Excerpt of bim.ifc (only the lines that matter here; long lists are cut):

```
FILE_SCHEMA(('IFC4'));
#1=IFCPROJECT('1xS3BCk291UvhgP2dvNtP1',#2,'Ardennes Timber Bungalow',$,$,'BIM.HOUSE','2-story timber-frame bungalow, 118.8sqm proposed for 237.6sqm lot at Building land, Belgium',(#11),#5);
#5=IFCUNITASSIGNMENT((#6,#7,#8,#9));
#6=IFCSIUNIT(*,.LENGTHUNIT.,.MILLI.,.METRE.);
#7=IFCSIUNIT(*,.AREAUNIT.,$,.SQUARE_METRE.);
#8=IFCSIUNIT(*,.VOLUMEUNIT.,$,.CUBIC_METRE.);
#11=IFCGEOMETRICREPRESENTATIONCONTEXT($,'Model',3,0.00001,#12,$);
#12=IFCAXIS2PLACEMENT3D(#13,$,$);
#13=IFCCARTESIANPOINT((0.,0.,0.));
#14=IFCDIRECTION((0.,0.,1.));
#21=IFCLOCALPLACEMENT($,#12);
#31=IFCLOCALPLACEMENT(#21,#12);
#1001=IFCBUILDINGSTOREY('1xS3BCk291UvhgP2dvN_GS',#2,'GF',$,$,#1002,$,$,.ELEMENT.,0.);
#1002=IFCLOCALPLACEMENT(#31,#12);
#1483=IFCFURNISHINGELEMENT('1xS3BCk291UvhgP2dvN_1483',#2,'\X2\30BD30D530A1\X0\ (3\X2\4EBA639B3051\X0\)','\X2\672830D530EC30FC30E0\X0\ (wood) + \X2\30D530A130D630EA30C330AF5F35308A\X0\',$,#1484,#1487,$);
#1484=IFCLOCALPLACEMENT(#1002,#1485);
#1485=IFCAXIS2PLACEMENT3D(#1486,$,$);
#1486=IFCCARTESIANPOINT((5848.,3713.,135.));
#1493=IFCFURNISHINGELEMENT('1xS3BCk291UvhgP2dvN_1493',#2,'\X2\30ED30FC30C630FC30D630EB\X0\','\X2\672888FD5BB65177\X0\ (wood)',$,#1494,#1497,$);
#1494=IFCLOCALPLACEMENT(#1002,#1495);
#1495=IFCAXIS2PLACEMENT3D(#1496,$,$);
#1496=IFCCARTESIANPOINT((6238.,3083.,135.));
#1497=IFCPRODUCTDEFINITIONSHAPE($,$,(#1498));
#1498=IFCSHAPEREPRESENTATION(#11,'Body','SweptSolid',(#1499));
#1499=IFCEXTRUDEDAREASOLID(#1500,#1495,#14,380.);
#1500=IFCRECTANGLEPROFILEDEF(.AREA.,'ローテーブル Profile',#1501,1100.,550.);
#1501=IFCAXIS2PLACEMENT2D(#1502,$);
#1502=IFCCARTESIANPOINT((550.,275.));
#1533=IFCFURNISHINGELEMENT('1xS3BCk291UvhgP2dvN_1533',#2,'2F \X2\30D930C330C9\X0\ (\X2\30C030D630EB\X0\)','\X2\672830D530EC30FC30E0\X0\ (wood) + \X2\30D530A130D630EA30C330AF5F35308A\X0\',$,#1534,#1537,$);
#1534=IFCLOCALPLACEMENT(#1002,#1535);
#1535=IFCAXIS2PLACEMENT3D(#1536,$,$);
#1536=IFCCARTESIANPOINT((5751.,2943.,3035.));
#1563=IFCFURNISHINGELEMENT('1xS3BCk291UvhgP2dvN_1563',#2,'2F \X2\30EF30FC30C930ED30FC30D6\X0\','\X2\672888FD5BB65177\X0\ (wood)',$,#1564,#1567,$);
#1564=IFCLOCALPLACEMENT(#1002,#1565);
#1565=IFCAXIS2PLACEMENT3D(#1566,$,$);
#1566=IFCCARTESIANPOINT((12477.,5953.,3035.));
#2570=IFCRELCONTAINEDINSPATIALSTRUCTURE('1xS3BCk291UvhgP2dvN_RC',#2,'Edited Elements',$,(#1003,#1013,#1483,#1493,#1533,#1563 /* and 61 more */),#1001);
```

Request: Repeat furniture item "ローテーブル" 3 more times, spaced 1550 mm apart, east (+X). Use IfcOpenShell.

```python
import numpy as np
import ifcopenshell
import ifcopenshell.api.geometry
import ifcopenshell.api.root
import ifcopenshell.util.element
import ifcopenshell.util.placement
import ifcopenshell.util.unit

model = ifcopenshell.open("bim.ifc")
unit_scale = ifcopenshell.util.unit.calculate_unit_scale(model)


def reuse_history(source, copy):
    """copy_class also copies each property set's owner history, people and application; keep the originals."""
    for rel in copy.IsDefinedBy:
        if rel.is_a("IfcRelDefinesByProperties") and (history := rel.RelatingPropertyDefinition.OwnerHistory):
            rel.RelatingPropertyDefinition.OwnerHistory = source.OwnerHistory
            ifcopenshell.util.element.remove_deep2(model, history)


source = model.by_guid("1xS3BCk291UvhgP2dvN_1493")
base = ifcopenshell.util.placement.get_local_placement(source.ObjectPlacement)
step = np.array([1.0, 0.0, 0.0]) * 1.55 / unit_scale

for i in range(1, 4):
    copy = ifcopenshell.api.root.copy_class(model, product=source)
    copy.Representation = ifcopenshell.util.element.copy_deep(
        model, source.Representation, exclude=["IfcGeometricRepresentationContext", "IfcRepresentationMap"]
    )
    reuse_history(source, copy)
    matrix = base.copy()
    matrix[:3, 3] += i * step
    print("added at", matrix[:3, 3].round(3) + 0.0)
    ifcopenshell.api.geometry.edit_object_placement(model, product=copy, matrix=matrix, is_si=False)

model.write("bim-out.ifc")
```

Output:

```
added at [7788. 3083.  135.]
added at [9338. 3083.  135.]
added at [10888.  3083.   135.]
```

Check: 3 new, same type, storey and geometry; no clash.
